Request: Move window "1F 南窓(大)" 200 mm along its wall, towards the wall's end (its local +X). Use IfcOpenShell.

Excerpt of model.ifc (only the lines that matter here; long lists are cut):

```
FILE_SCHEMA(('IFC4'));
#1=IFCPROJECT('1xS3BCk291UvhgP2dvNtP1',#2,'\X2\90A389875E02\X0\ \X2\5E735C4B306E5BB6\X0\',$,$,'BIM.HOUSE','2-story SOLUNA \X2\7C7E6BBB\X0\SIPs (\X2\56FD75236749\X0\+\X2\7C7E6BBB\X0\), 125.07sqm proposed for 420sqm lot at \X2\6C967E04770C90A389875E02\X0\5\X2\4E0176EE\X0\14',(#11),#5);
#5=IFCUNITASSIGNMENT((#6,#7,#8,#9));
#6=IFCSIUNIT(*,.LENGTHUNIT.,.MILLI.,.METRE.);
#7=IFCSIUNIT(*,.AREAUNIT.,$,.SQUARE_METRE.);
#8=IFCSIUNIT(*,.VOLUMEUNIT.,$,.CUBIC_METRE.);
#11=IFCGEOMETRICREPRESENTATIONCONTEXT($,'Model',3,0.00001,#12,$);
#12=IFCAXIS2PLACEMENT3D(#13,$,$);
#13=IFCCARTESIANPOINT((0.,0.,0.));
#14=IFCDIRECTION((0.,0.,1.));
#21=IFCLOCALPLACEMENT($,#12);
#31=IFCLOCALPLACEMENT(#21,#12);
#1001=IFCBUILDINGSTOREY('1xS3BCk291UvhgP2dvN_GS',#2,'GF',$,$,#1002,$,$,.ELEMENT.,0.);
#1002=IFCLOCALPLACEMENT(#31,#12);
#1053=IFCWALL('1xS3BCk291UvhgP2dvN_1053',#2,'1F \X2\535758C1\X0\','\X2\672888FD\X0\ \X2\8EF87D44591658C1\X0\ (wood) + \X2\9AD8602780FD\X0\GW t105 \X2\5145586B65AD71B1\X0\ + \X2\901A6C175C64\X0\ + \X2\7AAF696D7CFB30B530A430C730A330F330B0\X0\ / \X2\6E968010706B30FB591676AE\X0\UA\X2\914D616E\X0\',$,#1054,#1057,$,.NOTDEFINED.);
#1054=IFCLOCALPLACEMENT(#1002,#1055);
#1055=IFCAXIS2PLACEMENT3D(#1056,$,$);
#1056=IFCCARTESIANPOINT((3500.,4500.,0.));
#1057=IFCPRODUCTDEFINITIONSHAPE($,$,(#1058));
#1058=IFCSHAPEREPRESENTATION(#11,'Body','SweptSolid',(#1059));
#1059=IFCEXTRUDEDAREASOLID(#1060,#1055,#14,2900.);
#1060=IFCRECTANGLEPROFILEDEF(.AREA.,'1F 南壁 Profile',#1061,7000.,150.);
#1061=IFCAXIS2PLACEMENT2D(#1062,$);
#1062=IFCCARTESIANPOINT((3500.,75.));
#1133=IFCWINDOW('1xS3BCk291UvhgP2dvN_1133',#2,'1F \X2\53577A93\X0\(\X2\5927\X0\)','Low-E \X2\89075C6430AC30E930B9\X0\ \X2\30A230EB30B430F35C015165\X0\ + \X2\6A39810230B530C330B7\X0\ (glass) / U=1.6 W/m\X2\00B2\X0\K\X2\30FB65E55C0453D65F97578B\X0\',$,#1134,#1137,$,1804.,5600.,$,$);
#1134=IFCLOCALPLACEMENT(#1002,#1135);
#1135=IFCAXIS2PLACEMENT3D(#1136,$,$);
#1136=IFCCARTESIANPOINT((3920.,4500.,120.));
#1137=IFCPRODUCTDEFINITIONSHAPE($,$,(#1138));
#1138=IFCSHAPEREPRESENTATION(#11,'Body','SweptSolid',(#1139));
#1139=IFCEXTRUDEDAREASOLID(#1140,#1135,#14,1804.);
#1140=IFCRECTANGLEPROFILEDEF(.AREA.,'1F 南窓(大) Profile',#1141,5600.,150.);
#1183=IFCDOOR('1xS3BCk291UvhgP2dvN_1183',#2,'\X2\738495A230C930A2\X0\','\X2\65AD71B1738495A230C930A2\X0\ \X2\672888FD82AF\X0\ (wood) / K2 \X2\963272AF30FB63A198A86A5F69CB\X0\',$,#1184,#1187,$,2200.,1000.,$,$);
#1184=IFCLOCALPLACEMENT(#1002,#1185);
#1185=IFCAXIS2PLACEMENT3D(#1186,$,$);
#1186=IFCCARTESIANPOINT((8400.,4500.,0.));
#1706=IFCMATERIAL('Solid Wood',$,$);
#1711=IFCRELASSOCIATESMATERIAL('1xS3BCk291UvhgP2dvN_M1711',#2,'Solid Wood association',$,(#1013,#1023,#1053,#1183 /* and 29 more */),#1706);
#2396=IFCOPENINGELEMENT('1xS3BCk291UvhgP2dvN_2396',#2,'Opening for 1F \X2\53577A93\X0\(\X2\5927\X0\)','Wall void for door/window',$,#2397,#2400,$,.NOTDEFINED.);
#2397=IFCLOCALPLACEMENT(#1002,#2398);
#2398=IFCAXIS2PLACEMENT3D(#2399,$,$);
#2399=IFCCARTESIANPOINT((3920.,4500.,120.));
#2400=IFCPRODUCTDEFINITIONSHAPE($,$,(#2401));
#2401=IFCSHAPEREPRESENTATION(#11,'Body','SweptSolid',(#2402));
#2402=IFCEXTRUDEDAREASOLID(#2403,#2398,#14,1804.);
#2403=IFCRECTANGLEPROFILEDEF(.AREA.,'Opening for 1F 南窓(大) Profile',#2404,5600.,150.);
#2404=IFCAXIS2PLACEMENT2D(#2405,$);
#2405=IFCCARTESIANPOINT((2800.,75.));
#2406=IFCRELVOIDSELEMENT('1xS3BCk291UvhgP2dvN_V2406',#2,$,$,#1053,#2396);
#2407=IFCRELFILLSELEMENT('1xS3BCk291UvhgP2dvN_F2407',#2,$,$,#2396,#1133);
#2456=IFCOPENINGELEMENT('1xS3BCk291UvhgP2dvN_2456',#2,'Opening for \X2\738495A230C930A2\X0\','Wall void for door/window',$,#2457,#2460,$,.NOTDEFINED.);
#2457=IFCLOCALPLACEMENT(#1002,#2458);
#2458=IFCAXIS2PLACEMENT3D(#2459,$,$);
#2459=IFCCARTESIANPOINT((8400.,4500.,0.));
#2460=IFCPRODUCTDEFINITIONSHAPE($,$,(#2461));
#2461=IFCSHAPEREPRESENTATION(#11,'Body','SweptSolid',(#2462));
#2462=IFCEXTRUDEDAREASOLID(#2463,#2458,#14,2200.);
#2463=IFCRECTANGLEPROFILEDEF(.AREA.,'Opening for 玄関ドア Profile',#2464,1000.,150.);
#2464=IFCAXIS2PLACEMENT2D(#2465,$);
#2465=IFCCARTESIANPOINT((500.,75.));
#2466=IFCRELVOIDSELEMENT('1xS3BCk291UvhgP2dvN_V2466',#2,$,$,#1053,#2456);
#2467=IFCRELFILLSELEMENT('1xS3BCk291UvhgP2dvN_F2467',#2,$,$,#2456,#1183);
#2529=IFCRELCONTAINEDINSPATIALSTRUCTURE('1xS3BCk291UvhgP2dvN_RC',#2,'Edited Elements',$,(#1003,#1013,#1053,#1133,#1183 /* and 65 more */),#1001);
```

```python
import ifcopenshell
import ifcopenshell.api.geometry
import ifcopenshell.util.placement

model = ifcopenshell.open("model.ifc")

window = model.by_id(1133)
opening = window.FillsVoids[0].RelatingOpeningElement
wall = opening.VoidsElements[0].RelatingBuildingElement

wall_matrix = ifcopenshell.util.placement.get_local_placement(wall.ObjectPlacement)
shift = wall_matrix[:3, 0] * 200.0
before = ifcopenshell.util.placement.get_local_placement(window.ObjectPlacement)[:3, 3].copy()

# The window is not placed relative to its opening, so move both.
for product in (opening, window):
    matrix = ifcopenshell.util.placement.get_local_placement(product.ObjectPlacement)
    matrix[:3, 3] += shift
    ifcopenshell.api.geometry.edit_object_placement(model, product=product, matrix=matrix, is_si=False)

after = ifcopenshell.util.placement.get_local_placement(window.ObjectPlacement)[:3, 3]
print("window moved by", (after - before).round(3) + 0.0)

model.write("model-out.ifc")
```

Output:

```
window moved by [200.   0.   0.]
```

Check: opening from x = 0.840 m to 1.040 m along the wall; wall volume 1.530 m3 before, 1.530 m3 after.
